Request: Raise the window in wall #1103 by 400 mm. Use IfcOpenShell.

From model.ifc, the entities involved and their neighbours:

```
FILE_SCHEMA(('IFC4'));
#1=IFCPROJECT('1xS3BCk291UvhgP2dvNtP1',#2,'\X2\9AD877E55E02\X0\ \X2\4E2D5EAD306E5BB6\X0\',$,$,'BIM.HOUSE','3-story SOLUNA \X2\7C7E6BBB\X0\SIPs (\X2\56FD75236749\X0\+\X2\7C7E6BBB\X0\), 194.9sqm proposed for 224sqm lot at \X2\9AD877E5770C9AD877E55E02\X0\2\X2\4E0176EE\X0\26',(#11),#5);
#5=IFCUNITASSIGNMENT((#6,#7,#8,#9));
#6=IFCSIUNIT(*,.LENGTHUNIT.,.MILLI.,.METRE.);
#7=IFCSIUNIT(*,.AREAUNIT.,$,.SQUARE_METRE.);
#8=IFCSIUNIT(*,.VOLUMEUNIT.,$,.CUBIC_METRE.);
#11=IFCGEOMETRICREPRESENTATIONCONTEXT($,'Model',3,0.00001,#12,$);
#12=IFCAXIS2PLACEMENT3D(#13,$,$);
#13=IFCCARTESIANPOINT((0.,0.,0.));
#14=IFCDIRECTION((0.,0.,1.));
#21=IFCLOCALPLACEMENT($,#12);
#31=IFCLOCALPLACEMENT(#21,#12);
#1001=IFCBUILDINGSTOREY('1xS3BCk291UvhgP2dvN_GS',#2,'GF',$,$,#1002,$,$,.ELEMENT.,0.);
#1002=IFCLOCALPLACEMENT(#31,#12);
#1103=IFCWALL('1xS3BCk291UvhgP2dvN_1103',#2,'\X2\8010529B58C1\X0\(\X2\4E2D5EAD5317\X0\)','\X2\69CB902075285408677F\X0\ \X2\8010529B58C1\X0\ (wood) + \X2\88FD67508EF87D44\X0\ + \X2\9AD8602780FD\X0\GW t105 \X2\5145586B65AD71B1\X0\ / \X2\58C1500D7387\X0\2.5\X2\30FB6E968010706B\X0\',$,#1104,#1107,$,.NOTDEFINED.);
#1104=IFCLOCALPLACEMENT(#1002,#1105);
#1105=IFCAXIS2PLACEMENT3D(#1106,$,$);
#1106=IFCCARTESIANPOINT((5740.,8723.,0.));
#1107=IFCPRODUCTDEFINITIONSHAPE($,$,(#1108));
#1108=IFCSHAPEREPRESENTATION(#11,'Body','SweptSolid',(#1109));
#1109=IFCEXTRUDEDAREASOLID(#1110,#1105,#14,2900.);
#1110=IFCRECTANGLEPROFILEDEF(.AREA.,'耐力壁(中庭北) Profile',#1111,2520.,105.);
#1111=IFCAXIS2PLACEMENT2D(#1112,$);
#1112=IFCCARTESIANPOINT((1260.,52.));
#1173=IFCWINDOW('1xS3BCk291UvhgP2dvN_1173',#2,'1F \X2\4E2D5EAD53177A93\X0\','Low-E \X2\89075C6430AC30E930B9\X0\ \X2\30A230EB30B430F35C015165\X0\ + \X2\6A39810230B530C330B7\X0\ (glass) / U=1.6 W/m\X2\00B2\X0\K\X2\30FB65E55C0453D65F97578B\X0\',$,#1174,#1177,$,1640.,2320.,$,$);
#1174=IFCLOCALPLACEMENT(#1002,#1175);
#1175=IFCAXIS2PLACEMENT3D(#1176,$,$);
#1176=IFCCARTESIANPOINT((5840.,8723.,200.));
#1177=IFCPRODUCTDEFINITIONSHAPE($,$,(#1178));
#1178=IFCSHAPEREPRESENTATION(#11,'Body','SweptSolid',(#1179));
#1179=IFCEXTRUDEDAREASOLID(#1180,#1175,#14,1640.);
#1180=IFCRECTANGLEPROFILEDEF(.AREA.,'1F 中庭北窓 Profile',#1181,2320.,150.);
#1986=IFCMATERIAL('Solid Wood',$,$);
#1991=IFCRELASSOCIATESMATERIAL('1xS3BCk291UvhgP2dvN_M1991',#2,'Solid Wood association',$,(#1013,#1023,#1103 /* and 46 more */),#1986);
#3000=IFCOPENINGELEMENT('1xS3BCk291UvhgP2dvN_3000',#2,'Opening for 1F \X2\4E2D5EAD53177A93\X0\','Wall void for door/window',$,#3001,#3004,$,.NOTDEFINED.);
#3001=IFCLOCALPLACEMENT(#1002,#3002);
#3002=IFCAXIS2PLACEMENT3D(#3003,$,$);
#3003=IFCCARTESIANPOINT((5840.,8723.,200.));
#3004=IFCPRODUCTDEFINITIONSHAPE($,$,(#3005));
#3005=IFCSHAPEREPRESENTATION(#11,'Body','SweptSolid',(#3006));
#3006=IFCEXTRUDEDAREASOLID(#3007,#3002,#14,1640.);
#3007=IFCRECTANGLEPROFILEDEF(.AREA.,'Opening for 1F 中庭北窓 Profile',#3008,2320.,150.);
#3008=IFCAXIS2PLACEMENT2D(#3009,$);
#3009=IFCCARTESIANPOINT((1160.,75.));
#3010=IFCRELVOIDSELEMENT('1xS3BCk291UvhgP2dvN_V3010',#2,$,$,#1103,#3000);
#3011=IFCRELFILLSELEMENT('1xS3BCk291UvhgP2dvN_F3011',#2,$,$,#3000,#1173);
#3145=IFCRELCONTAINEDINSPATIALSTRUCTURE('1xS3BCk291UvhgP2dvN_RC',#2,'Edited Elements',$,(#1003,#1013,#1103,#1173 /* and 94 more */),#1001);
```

```python
import numpy as np
import ifcopenshell
import ifcopenshell.api.geometry
import ifcopenshell.util.placement
import ifcopenshell.util.unit

model = ifcopenshell.open("model.ifc")
unit_scale = ifcopenshell.util.unit.calculate_unit_scale(model)

window = model.by_guid("1xS3BCk291UvhgP2dvN_1173")
opening = window.FillsVoids[0].RelatingOpeningElement
dz = 400.0

shift = np.array([0.0, 0.0, dz])
# The window is not placed relative to its opening, so move both.
for product in (opening, window):
    matrix = ifcopenshell.util.placement.get_local_placement(product.ObjectPlacement)
    matrix[:3, 3] += shift
    ifcopenshell.api.geometry.edit_object_placement(model, product=product, matrix=matrix, is_si=False)

print(f"moved by {dz * unit_scale:+.3f} m")

model.write("model_rev.ifc")
```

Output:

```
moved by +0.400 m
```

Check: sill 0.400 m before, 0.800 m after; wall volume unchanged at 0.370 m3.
